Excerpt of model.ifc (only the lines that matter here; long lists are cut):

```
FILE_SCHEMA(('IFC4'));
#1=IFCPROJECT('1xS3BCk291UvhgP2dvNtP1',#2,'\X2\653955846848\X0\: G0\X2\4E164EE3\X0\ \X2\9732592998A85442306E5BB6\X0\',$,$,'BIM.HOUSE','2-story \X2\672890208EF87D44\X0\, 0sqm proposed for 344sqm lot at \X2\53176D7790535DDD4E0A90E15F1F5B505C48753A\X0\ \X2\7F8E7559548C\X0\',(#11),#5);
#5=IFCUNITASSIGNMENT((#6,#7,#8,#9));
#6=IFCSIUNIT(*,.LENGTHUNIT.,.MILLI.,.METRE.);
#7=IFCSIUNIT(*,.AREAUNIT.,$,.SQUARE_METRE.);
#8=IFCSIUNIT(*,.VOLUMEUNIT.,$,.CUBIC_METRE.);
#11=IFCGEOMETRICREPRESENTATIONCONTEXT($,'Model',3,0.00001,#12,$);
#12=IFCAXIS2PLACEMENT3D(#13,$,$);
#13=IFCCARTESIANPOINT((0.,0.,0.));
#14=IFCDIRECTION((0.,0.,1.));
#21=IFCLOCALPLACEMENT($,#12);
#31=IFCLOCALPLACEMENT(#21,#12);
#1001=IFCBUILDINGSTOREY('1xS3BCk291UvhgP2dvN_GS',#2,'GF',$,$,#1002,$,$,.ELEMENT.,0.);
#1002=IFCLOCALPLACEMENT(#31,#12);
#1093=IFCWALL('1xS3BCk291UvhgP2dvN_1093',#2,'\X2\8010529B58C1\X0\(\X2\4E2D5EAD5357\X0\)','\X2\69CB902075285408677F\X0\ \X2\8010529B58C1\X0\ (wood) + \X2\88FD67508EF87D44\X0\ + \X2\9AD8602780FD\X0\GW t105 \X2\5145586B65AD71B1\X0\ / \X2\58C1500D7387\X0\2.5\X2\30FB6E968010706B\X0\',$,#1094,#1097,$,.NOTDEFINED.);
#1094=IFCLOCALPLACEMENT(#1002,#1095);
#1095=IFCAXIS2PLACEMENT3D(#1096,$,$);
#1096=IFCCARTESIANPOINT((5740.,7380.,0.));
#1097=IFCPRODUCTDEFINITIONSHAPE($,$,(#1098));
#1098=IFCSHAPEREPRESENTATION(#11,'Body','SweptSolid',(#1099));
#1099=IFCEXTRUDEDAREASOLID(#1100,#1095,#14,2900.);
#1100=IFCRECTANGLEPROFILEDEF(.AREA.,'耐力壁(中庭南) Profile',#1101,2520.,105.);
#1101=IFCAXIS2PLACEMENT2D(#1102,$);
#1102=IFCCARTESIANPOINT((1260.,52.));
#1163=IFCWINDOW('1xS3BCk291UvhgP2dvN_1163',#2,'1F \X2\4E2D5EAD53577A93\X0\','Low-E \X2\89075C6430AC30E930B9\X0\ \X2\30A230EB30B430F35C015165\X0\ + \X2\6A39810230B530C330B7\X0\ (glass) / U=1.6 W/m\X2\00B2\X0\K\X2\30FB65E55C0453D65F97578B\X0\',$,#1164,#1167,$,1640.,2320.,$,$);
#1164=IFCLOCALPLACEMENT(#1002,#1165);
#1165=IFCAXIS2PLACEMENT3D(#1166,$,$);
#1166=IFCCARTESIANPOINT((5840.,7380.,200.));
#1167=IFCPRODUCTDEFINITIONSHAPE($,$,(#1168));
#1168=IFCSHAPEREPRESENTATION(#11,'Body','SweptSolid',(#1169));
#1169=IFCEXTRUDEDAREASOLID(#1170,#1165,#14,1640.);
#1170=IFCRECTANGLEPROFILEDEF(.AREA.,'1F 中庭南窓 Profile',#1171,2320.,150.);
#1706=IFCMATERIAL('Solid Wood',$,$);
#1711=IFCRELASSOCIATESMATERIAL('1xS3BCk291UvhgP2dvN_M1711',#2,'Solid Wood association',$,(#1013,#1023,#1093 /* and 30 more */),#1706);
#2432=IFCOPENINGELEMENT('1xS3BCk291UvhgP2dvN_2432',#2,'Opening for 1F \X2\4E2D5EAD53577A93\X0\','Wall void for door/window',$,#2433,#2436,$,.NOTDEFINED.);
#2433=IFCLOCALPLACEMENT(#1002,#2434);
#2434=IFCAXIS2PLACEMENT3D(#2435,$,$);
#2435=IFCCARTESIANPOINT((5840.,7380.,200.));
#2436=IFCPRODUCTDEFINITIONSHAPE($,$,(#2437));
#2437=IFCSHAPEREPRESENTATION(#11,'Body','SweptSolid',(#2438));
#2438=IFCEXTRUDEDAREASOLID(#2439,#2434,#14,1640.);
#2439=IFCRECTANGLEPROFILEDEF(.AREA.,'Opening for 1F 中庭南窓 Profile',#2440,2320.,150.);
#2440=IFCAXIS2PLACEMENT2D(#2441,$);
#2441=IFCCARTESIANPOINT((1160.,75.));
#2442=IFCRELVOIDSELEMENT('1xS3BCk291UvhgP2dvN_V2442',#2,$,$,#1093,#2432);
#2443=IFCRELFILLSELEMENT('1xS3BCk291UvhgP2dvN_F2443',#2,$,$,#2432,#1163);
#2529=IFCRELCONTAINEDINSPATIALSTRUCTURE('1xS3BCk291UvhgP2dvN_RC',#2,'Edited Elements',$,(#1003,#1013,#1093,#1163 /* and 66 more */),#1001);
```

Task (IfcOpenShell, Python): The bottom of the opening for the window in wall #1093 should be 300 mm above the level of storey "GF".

```python
import numpy as np
import ifcopenshell
import ifcopenshell.api.geometry
import ifcopenshell.geom
import ifcopenshell.util.element
import ifcopenshell.util.placement
import ifcopenshell.util.shape
import ifcopenshell.util.unit

model = ifcopenshell.open("model.ifc")
unit_scale = ifcopenshell.util.unit.calculate_unit_scale(model)

window = model.by_guid("1xS3BCk291UvhgP2dvN_1163")
opening = window.FillsVoids[0].RelatingOpeningElement
storey = ifcopenshell.util.element.get_container(window, ifc_class="IfcBuildingStorey")
level = ifcopenshell.util.placement.get_local_placement(storey.ObjectPlacement)[2, 3]

# The opening's origin need not be at the sill, so measure its lowest point.
shape = ifcopenshell.geom.create_shape(ifcopenshell.geom.settings(), opening)
bottom = ifcopenshell.util.shape.get_shape_bottom_elevation(shape, shape.geometry) / unit_scale
dz = level + 300.0 - bottom

shift = np.array([0.0, 0.0, dz])
# The window is not placed relative to its opening, so move both.
for product in (opening, window):
    matrix = ifcopenshell.util.placement.get_local_placement(product.ObjectPlacement)
    matrix[:3, 3] += shift
    ifcopenshell.api.geometry.edit_object_placement(model, product=product, matrix=matrix, is_si=False)

print(f"moved by {dz * unit_scale:+.3f} m")

model.write("model_rev.ifc")
```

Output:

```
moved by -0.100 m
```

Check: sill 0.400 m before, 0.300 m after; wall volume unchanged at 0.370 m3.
